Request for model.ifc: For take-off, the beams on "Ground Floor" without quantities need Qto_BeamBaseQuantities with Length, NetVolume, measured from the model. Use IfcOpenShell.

First a look at what the model holds.

```python
import ifcopenshell
import ifcopenshell.util.element
import ifcopenshell.util.unit

model = ifcopenshell.open("model.ifc")
print(model.schema)
for unit_type in ("LENGTHUNIT", "AREAUNIT", "VOLUMEUNIT"):
    print(unit_type, ifcopenshell.util.unit.calculate_unit_scale(model, unit_type))
storey = next(s for s in model.by_type("IfcBuildingStorey") if s.Name == "Ground Floor")
beams = [e for e in ifcopenshell.util.element.get_decomposition(storey) if e.is_a("IfcBeam")]
for e in sorted(beams, key=lambda e: e.id()):
    print(e.id(), e.is_a(), e.Name, list(ifcopenshell.util.element.get_psets(e, qtos_only=True)), sep=" | ")
```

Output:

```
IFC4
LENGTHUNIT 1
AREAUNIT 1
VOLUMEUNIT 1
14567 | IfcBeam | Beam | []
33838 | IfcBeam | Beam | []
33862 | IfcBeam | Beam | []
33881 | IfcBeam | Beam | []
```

```python
import ifcopenshell
import ifcopenshell.api.pset
import ifcopenshell.geom
import ifcopenshell.util.element
import ifcopenshell.util.shape
import ifcopenshell.util.unit

model = ifcopenshell.open("model.ifc")
unit_scale = ifcopenshell.util.unit.calculate_unit_scale(model)
volume_scale = ifcopenshell.util.unit.calculate_unit_scale(model, "VOLUMEUNIT")
settings = ifcopenshell.geom.settings()

storey = next(s for s in model.by_type("IfcBuildingStorey") if s.Name == "Ground Floor")
beams = [e for e in ifcopenshell.util.element.get_decomposition(storey) if e.is_a("IfcBeam")]

for e in sorted(beams, key=lambda e: e.id()):
    if ifcopenshell.util.element.get_psets(e, qtos_only=True, should_inherit=False):
        continue
    # Geometry comes back in metres, in the element's own axes.
    shape = ifcopenshell.geom.create_shape(settings, e)
    values = {
        "Length": ifcopenshell.util.shape.get_max_xyz(shape.geometry) / unit_scale,
        "NetVolume": ifcopenshell.util.shape.get_volume(shape.geometry) / volume_scale,
    }
    qto = ifcopenshell.api.pset.add_qto(model, product=e, name="Qto_BeamBaseQuantities")
    ifcopenshell.api.pset.edit_qto(model, qto=qto, properties=values)
    print(e.id(), {k: round(v, 3) for k, v in values.items()})

model.write("model_v2.ifc")
```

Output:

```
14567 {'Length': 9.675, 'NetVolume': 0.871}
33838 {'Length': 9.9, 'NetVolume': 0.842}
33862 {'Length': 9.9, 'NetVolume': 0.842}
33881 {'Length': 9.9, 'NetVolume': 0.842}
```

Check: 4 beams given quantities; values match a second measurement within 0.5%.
